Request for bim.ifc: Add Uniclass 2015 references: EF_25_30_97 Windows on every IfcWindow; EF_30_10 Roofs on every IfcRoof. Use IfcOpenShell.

First a look at what the model holds.

```python
import ifcopenshell

model = ifcopenshell.open("bim.ifc")
print(model.schema)
print("classifications:", [c.Name for c in model.by_type("IfcClassification")])
for ifc_class in ("IfcDoor", "IfcRoof", "IfcStair", "IfcWall", "IfcWindow"):
    print(ifc_class, len(model.by_type(ifc_class)))
```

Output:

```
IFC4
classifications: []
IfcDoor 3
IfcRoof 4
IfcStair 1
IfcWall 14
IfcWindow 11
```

```python
import ifcopenshell
import ifcopenshell.api.classification

model = ifcopenshell.open("bim.ifc")

system = ifcopenshell.api.classification.add_classification(model, classification="Uniclass 2015")

codes = {
    "IfcWindow": ("EF_25_30_97", "Windows"),
    "IfcRoof": ("EF_30_10", "Roofs"),
}
for ifc_class, (code, name) in codes.items():
    products = model.by_type(ifc_class)
    ifcopenshell.api.classification.add_reference(
        model, products=products, classification=system, identification=code, name=name
    )
    print(code, len(products))

model.write("bim_rev.ifc")
```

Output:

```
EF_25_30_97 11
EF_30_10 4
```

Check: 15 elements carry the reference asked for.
